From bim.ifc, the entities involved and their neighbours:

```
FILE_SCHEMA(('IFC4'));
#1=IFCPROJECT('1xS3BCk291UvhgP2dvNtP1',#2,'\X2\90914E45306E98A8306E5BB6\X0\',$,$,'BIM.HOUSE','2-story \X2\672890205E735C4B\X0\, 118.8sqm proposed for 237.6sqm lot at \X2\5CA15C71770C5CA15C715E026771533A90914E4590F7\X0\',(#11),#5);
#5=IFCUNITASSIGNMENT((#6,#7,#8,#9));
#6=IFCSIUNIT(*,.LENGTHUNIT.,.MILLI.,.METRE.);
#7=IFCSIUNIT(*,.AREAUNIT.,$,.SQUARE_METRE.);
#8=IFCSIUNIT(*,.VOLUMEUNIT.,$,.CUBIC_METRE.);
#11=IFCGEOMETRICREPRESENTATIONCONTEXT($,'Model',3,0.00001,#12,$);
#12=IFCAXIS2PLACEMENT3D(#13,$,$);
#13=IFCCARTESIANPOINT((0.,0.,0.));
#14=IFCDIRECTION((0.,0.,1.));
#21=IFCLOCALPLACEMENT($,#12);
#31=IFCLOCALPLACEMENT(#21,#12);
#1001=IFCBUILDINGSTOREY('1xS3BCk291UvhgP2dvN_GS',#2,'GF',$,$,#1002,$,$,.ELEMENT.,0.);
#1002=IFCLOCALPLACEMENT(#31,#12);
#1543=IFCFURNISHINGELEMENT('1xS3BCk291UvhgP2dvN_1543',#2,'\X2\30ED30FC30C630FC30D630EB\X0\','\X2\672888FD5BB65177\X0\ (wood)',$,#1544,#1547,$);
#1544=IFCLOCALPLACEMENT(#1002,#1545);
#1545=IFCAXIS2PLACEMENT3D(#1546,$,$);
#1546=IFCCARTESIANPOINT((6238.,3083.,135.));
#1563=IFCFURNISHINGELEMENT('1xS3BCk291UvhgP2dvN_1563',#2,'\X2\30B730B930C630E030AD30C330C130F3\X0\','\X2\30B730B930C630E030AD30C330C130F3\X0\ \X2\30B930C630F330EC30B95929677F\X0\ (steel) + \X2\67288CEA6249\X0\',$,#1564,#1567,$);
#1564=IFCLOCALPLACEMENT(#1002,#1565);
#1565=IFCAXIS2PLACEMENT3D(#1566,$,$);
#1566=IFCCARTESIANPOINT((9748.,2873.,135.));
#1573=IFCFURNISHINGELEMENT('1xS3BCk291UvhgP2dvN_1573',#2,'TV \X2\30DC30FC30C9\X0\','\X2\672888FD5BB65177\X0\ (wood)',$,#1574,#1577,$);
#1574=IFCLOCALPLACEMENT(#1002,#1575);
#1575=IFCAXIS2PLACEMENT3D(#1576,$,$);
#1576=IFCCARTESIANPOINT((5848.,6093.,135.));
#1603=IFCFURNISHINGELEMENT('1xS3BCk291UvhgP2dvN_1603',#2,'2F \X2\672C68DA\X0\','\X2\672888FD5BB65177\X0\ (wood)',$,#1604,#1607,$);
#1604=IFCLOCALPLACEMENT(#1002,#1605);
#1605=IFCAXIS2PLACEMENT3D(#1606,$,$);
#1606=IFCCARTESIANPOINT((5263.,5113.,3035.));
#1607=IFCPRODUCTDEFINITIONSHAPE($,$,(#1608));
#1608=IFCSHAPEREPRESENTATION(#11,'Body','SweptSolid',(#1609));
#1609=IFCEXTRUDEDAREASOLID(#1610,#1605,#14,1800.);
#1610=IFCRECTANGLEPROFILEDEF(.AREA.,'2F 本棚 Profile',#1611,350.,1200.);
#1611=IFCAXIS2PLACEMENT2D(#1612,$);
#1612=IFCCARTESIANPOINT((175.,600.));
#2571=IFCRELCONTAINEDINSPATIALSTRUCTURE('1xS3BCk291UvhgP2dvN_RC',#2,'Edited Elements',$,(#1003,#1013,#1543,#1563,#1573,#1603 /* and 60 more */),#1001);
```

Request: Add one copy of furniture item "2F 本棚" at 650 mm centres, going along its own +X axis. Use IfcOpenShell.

```python
import ifcopenshell
import ifcopenshell.api.geometry
import ifcopenshell.api.root
import ifcopenshell.util.element
import ifcopenshell.util.placement

model = ifcopenshell.open("bim.ifc")


def reuse_history(source, copy):
    """copy_class also copies each property set's owner history, people and application; keep the originals."""
    for rel in copy.IsDefinedBy:
        if rel.is_a("IfcRelDefinesByProperties") and (history := rel.RelatingPropertyDefinition.OwnerHistory):
            rel.RelatingPropertyDefinition.OwnerHistory = source.OwnerHistory
            ifcopenshell.util.element.remove_deep2(model, history)


source = model.by_id(1603)
base = ifcopenshell.util.placement.get_local_placement(source.ObjectPlacement)
step = base[:3, 0] * 650.0

for i in range(1, 2):
    copy = ifcopenshell.api.root.copy_class(model, product=source)
    copy.Representation = ifcopenshell.util.element.copy_deep(
        model, source.Representation, exclude=["IfcGeometricRepresentationContext", "IfcRepresentationMap"]
    )
    reuse_history(source, copy)
    matrix = base.copy()
    matrix[:3, 3] += i * step
    print("added at", matrix[:3, 3].round(3) + 0.0)
    ifcopenshell.api.geometry.edit_object_placement(model, product=copy, matrix=matrix, is_si=False)

model.write("bim_rev.ifc")
```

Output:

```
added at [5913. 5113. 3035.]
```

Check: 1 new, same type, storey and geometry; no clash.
